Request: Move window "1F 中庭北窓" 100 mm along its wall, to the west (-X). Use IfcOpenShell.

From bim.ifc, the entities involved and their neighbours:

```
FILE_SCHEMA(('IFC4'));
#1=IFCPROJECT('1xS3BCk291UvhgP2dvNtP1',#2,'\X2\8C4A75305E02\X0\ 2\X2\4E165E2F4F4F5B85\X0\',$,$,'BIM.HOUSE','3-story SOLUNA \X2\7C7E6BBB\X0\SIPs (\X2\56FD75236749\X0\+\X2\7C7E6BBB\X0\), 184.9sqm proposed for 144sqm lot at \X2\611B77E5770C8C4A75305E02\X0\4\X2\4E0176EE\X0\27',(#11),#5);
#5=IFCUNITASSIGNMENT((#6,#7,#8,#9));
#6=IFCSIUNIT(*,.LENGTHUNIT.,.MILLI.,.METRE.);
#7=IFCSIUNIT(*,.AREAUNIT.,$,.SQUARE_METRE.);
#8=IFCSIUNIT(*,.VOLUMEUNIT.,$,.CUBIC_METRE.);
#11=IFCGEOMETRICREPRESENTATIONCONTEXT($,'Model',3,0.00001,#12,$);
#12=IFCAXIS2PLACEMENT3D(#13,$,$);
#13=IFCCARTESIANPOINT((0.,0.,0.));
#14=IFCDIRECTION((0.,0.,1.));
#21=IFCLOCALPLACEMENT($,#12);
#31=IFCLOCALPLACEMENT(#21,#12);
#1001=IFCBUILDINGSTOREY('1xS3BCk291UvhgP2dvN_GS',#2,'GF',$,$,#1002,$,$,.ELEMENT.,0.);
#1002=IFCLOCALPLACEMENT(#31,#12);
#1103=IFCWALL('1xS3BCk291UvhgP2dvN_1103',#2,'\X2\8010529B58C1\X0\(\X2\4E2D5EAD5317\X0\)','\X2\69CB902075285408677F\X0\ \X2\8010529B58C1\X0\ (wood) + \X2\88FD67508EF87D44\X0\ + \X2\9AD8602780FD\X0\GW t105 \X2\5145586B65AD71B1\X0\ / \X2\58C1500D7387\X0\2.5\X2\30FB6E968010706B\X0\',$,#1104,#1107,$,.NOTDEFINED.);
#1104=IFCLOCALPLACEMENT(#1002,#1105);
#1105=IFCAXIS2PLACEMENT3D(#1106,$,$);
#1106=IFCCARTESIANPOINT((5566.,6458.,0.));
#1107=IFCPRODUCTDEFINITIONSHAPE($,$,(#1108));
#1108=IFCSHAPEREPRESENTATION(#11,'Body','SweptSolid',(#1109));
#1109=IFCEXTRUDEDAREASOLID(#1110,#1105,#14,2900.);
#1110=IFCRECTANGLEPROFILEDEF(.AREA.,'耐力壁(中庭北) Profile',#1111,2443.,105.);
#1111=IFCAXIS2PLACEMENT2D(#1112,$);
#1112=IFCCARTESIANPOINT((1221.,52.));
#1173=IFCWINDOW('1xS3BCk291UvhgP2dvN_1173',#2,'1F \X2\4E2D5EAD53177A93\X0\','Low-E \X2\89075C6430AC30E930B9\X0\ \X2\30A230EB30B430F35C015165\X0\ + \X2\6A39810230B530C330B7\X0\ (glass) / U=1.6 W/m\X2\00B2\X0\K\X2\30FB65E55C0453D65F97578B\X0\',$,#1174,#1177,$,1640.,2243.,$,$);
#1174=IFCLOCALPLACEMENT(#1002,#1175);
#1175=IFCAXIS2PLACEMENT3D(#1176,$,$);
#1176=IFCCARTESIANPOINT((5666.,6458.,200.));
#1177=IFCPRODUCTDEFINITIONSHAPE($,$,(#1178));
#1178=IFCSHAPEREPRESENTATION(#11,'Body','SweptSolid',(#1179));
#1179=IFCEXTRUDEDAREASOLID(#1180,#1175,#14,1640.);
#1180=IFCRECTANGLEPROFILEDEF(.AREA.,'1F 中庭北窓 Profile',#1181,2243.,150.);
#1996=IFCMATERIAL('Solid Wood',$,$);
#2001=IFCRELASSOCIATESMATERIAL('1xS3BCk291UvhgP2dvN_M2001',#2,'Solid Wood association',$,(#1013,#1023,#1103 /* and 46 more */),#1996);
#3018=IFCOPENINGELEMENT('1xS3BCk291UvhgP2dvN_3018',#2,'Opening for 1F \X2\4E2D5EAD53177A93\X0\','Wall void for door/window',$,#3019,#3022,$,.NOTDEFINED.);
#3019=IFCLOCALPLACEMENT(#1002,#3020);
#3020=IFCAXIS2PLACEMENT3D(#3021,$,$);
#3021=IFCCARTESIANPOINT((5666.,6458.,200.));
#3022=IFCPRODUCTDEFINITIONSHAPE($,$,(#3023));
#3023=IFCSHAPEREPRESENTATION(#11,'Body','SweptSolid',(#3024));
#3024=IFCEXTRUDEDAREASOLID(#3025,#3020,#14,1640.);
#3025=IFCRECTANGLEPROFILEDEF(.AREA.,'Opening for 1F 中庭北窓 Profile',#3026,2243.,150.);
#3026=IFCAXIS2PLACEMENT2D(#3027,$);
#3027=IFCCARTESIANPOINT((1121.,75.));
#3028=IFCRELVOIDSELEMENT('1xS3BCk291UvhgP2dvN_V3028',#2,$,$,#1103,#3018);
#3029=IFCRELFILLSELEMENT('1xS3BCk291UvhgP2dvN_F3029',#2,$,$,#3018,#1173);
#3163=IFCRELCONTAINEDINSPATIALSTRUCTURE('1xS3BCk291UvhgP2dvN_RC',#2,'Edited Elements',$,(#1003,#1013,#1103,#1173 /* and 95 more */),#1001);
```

```python
import ifcopenshell
import ifcopenshell.api.geometry
import ifcopenshell.util.placement
import ifcopenshell.util.unit

model = ifcopenshell.open("bim.ifc")
unit_scale = ifcopenshell.util.unit.calculate_unit_scale(model)

window = model.by_id(1173)
opening = window.FillsVoids[0].RelatingOpeningElement
wall = opening.VoidsElements[0].RelatingBuildingElement

wall_matrix = ifcopenshell.util.placement.get_local_placement(wall.ObjectPlacement)
shift = wall_matrix[:3, 0] * -0.1 / unit_scale
before = ifcopenshell.util.placement.get_local_placement(window.ObjectPlacement)[:3, 3].copy()

# The window is not placed relative to its opening, so move both.
for product in (opening, window):
    matrix = ifcopenshell.util.placement.get_local_placement(product.ObjectPlacement)
    matrix[:3, 3] += shift
    ifcopenshell.api.geometry.edit_object_placement(model, product=product, matrix=matrix, is_si=False)

after = ifcopenshell.util.placement.get_local_placement(window.ObjectPlacement)[:3, 3]
print("window moved by", (after - before).round(3) + 0.0)

model.write("bim-out.ifc")
```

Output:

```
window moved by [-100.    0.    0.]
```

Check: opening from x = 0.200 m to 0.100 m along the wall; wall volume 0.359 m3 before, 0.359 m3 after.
